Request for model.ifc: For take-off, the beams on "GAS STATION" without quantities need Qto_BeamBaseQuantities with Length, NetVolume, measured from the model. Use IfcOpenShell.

First a look at what the model holds.

```python
import ifcopenshell
import ifcopenshell.util.element
import ifcopenshell.util.unit

model = ifcopenshell.open("model.ifc")
print(model.schema)
for unit_type in ("LENGTHUNIT", "AREAUNIT", "VOLUMEUNIT"):
    print(unit_type, ifcopenshell.util.unit.calculate_unit_scale(model, unit_type))
storey = next(s for s in model.by_type("IfcBuildingStorey") if s.Name == "GAS STATION")
beams = [e for e in ifcopenshell.util.element.get_decomposition(storey) if e.is_a("IfcBeam")]
for e in sorted(beams, key=lambda e: e.id()):
    print(e.id(), e.is_a(), e.Name, list(ifcopenshell.util.element.get_psets(e, qtos_only=True)), sep=" | ")
```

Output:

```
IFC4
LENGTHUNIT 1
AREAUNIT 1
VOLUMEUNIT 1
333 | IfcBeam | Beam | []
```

```python
import ifcopenshell
import ifcopenshell.api.pset
import ifcopenshell.geom
import ifcopenshell.util.element
import ifcopenshell.util.shape
import ifcopenshell.util.unit

model = ifcopenshell.open("model.ifc")
unit_scale = ifcopenshell.util.unit.calculate_unit_scale(model)
volume_scale = ifcopenshell.util.unit.calculate_unit_scale(model, "VOLUMEUNIT")
settings = ifcopenshell.geom.settings()

storey = next(s for s in model.by_type("IfcBuildingStorey") if s.Name == "GAS STATION")
beams = [e for e in ifcopenshell.util.element.get_decomposition(storey) if e.is_a("IfcBeam")]

for e in sorted(beams, key=lambda e: e.id()):
    if ifcopenshell.util.element.get_psets(e, qtos_only=True, should_inherit=False):
        continue
    # Geometry comes back in metres, in the element's own axes.
    shape = ifcopenshell.geom.create_shape(settings, e)
    values = {
        "Length": ifcopenshell.util.shape.get_max_xyz(shape.geometry) / unit_scale,
        "NetVolume": ifcopenshell.util.shape.get_volume(shape.geometry) / volume_scale,
    }
    qto = ifcopenshell.api.pset.add_qto(model, product=e, name="Qto_BeamBaseQuantities")
    ifcopenshell.api.pset.edit_qto(model, qto=qto, properties=values)
    print(e.id(), {k: round(v, 3) for k, v in values.items()})

model.write("model-out.ifc")
```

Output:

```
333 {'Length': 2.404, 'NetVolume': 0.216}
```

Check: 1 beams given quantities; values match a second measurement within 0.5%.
